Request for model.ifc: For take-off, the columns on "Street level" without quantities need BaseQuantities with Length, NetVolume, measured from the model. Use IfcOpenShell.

First a look at what the model holds.

```python
import ifcopenshell
import ifcopenshell.util.element
import ifcopenshell.util.unit

model = ifcopenshell.open("model.ifc")
print(model.schema)
for unit_type in ("LENGTHUNIT", "AREAUNIT", "VOLUMEUNIT"):
    print(unit_type, ifcopenshell.util.unit.calculate_unit_scale(model, unit_type))
storey = next(s for s in model.by_type("IfcBuildingStorey") if s.Name == "Street level")
columns = [e for e in ifcopenshell.util.element.get_decomposition(storey) if e.is_a("IfcColumn")]
for e in sorted(columns, key=lambda e: e.id()):
    print(e.id(), e.is_a(), e.Name, list(ifcopenshell.util.element.get_psets(e, qtos_only=True)), sep=" | ")
```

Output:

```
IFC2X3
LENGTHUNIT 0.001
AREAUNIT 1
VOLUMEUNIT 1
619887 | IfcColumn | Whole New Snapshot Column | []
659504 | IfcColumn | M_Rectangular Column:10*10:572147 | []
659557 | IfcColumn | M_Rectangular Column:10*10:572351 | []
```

```python
import ifcopenshell
import ifcopenshell.api.pset
import ifcopenshell.geom
import ifcopenshell.util.element
import ifcopenshell.util.shape
import ifcopenshell.util.unit

model = ifcopenshell.open("model.ifc")
unit_scale = ifcopenshell.util.unit.calculate_unit_scale(model)
volume_scale = ifcopenshell.util.unit.calculate_unit_scale(model, "VOLUMEUNIT")
settings = ifcopenshell.geom.settings()

storey = next(s for s in model.by_type("IfcBuildingStorey") if s.Name == "Street level")
columns = [e for e in ifcopenshell.util.element.get_decomposition(storey) if e.is_a("IfcColumn")]

for e in sorted(columns, key=lambda e: e.id()):
    if ifcopenshell.util.element.get_psets(e, qtos_only=True, should_inherit=False):
        continue
    # Geometry comes back in metres, in the element's own axes.
    shape = ifcopenshell.geom.create_shape(settings, e)
    values = {
        "Length": ifcopenshell.util.shape.get_z(shape.geometry) / unit_scale,
        "NetVolume": ifcopenshell.util.shape.get_volume(shape.geometry) / volume_scale,
    }
    qto = ifcopenshell.api.pset.add_qto(model, product=e, name="BaseQuantities")
    ifcopenshell.api.pset.edit_qto(model, qto=qto, properties=values)
    print(e.id(), {k: round(v, 3) for k, v in values.items()})

model.write("model_edited.ifc")
```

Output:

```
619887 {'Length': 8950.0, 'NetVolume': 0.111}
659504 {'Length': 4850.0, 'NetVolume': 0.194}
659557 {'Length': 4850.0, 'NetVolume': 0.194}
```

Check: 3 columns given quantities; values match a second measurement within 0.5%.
